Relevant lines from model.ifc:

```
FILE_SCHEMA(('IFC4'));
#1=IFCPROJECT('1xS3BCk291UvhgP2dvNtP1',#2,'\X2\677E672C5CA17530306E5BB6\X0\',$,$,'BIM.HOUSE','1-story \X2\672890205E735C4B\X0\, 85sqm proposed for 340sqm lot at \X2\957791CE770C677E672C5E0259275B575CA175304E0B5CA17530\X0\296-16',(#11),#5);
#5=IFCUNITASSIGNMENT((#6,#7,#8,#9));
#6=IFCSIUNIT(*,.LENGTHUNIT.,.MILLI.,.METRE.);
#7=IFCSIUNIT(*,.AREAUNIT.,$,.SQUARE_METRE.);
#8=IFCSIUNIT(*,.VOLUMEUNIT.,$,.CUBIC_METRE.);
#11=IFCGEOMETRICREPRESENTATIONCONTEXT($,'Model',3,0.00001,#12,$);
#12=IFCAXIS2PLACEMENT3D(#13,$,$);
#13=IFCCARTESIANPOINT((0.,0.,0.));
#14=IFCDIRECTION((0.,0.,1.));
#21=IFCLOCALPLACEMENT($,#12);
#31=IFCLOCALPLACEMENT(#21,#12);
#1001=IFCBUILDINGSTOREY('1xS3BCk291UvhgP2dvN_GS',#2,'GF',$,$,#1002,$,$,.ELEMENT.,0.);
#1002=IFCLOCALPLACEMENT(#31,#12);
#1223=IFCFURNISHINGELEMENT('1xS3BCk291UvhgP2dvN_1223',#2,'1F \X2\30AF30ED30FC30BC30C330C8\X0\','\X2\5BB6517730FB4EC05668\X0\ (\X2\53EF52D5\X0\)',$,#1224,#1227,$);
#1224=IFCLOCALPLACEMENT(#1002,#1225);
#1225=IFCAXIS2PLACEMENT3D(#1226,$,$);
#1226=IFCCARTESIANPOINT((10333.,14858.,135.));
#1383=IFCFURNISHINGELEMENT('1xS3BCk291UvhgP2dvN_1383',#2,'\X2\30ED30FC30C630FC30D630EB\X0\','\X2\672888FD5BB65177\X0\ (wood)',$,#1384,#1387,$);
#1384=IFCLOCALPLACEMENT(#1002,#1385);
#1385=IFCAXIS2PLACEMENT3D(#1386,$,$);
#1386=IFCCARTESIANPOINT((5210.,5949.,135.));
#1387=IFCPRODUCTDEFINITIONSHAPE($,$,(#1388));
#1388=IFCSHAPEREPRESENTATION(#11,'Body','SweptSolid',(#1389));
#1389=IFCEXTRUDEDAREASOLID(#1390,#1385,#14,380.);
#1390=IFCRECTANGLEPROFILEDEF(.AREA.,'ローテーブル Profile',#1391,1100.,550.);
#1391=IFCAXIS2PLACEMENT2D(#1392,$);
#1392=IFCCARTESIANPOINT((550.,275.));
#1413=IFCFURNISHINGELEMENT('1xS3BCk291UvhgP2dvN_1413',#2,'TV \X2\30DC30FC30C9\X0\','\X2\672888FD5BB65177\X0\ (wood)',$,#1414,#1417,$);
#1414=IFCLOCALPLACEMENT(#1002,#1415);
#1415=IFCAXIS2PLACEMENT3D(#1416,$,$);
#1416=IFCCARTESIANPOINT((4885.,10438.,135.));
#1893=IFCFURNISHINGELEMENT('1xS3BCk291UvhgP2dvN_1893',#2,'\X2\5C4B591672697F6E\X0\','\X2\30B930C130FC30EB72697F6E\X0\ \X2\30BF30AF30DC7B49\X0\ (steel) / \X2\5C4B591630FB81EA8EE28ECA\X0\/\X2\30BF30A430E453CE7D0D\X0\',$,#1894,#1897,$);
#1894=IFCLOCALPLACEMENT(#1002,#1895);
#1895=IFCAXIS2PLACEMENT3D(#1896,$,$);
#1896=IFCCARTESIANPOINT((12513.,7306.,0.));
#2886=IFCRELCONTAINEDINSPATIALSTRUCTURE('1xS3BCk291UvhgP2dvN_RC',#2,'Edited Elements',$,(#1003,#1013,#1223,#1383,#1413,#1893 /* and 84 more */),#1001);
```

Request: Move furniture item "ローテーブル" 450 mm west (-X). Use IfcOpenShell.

```python
import ifcopenshell
import ifcopenshell.api.geometry
import ifcopenshell.util.placement

model = ifcopenshell.open("model.ifc")

item = model.by_guid("1xS3BCk291UvhgP2dvN_1383")
matrix = ifcopenshell.util.placement.get_local_placement(item.ObjectPlacement)
matrix[0, 3] -= 450.0
ifcopenshell.api.geometry.edit_object_placement(model, product=item, matrix=matrix, is_si=False)

print(ifcopenshell.util.placement.get_local_placement(item.ObjectPlacement).round(3) + 0.0)

model.write("model-out.ifc")
```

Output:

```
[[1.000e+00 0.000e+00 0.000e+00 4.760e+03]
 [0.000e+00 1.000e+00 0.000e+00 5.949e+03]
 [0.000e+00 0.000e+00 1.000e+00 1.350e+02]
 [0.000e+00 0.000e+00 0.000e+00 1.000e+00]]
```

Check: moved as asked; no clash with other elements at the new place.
